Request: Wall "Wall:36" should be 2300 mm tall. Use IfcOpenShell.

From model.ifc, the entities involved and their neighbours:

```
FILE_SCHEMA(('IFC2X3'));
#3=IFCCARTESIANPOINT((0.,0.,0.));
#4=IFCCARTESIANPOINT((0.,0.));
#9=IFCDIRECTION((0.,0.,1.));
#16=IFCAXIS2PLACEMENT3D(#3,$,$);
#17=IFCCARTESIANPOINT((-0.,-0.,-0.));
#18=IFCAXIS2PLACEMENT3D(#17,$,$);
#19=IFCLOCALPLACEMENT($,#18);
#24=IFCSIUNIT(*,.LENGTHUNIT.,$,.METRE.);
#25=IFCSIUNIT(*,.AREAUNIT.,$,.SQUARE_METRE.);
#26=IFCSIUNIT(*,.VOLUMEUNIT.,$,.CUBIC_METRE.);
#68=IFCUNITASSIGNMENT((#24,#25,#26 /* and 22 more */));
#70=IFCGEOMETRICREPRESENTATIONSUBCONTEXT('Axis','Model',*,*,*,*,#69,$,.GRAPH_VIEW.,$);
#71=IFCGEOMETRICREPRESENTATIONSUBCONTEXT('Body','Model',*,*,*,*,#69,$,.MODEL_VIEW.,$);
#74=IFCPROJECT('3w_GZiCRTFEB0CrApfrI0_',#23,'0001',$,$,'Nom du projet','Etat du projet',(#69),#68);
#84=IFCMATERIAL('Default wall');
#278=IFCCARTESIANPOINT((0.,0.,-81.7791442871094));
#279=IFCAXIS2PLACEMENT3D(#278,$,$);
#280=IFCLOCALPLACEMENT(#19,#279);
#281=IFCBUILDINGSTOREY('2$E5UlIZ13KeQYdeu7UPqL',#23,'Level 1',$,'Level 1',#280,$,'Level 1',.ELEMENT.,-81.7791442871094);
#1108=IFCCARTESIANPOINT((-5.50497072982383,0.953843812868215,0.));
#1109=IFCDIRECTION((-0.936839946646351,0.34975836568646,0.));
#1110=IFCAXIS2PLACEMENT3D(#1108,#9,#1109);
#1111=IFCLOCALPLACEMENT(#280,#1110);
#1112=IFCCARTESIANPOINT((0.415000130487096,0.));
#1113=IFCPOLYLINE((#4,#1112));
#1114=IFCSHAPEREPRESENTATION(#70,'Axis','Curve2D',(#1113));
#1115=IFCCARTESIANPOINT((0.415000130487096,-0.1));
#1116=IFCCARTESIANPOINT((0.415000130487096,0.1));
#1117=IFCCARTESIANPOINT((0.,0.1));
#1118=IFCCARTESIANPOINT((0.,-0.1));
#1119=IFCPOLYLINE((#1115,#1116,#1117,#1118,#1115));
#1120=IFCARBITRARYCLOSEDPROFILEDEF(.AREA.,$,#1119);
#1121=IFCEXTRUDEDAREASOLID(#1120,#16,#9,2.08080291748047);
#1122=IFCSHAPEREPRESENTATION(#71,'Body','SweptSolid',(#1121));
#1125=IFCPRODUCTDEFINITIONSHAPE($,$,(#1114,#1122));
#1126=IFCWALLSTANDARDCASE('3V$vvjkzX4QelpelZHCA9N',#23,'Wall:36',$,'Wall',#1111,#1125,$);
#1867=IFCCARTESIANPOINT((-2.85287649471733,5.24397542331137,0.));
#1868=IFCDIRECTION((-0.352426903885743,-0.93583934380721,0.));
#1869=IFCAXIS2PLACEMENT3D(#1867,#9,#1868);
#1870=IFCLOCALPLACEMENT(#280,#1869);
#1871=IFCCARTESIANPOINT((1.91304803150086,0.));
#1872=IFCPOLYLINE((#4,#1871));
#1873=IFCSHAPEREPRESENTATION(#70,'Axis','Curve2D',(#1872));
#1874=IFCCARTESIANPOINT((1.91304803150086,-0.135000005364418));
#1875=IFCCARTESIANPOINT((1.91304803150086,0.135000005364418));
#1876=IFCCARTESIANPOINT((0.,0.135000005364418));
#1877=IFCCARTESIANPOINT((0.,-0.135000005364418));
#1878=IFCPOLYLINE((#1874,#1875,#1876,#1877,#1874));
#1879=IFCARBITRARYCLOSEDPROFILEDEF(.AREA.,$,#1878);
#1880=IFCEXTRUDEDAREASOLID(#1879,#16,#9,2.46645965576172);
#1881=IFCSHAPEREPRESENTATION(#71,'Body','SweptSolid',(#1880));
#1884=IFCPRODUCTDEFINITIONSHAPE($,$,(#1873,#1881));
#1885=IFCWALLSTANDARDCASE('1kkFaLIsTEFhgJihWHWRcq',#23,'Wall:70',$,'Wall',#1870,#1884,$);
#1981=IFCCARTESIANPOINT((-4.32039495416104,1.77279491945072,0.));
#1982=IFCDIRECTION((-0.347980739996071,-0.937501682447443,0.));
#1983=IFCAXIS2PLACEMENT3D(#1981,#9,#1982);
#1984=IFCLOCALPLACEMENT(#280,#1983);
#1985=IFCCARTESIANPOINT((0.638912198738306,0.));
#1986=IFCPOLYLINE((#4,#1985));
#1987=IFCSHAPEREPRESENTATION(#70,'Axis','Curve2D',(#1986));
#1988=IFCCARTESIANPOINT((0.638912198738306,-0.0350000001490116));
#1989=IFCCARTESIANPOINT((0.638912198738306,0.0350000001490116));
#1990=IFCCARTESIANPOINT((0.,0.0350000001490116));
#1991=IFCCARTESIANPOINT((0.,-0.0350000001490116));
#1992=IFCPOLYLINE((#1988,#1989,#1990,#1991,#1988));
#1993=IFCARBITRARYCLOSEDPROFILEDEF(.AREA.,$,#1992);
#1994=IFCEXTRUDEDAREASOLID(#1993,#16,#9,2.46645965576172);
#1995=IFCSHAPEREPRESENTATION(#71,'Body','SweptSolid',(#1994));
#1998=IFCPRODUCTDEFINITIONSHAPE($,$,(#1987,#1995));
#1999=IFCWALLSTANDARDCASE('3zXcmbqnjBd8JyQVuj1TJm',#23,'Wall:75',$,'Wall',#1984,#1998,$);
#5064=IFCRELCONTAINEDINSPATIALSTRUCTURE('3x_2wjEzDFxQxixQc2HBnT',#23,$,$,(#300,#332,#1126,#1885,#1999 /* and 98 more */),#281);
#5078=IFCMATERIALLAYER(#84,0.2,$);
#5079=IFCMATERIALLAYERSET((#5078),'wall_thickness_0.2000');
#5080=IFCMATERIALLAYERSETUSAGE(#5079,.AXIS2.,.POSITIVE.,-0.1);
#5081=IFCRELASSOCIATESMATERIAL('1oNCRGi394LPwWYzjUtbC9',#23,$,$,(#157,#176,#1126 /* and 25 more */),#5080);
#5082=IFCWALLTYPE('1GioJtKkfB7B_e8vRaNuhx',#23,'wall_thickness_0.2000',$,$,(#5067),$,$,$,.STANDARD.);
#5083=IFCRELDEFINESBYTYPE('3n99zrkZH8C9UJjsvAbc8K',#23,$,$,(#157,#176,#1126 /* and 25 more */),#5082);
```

```python
import ifcopenshell
import ifcopenshell.geom
import ifcopenshell.util.representation
import ifcopenshell.util.shape
import ifcopenshell.util.unit

model = ifcopenshell.open("model.ifc")
unit_scale = ifcopenshell.util.unit.calculate_unit_scale(model)
settings = ifcopenshell.geom.settings()


def volume(element):
    """Net volume in cubic metres, openings subtracted."""
    shape = ifcopenshell.geom.create_shape(settings, element)
    return ifcopenshell.util.shape.get_volume(shape.geometry)


wall = model.by_guid("3V$vvjkzX4QelpelZHCA9N")
before = volume(wall)

body = ifcopenshell.util.representation.get_representation(wall, "Model", "Body")
solid = body.Items[0]
old_height = solid.Depth
solid.Depth = 2.3 / unit_scale
after = volume(wall)

print(f"height {old_height:g} -> {solid.Depth:g}, volume {before:.3f} -> {after:.3f} m3")

model.write("model_edited.ifc")
```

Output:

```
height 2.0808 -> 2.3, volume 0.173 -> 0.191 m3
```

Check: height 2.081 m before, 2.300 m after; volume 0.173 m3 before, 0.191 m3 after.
